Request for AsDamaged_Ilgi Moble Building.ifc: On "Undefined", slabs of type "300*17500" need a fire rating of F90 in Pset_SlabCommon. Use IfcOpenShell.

First a look at what the model holds.

```python
import ifcopenshell
import ifcopenshell.util.element

model = ifcopenshell.open("AsDamaged_Ilgi Moble Building.ifc")
print(model.schema)
storey = next(s for s in model.by_type("IfcBuildingStorey") if s.Name == "Undefined")
slabs = [e for e in ifcopenshell.util.element.get_decomposition(storey) if e.is_a("IfcSlab")]
seen = {}
for e in slabs:
    element_type = ifcopenshell.util.element.get_type(e)
    key = (element_type.Name if element_type != e and element_type else None, ifcopenshell.util.element.get_pset(e, "Pset_SlabCommon", "FireRating"))
    seen[key] = seen.get(key, 0) + 1
for (name, value), count in sorted(seen.items(), key=str):
    print(count, "x", name, "|", value)
```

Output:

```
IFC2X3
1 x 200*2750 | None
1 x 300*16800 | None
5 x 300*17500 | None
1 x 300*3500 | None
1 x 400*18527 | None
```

```python
import ifcopenshell
import ifcopenshell.api.pset
import ifcopenshell.util.element

model = ifcopenshell.open("AsDamaged_Ilgi Moble Building.ifc")

storey = next(s for s in model.by_type("IfcBuildingStorey") if s.Name == "Undefined")
slabs = [e for e in ifcopenshell.util.element.get_decomposition(storey) if e.is_a("IfcSlab")]

count = 0
for e in slabs:
    element_type = ifcopenshell.util.element.get_type(e)
    if element_type in (None, e) or element_type.Name != "300*17500":
        continue
    # add_pset returns the element's existing set when there is one.
    pset = ifcopenshell.api.pset.add_pset(model, product=e, name="Pset_SlabCommon")
    ifcopenshell.api.pset.edit_pset(model, pset=pset, properties={"FireRating": "F90"})
    count += 1

print(count, "slabs updated")

model.write("AsDamaged_Ilgi Moble Building_edited.ifc")
```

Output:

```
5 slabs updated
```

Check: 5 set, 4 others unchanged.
